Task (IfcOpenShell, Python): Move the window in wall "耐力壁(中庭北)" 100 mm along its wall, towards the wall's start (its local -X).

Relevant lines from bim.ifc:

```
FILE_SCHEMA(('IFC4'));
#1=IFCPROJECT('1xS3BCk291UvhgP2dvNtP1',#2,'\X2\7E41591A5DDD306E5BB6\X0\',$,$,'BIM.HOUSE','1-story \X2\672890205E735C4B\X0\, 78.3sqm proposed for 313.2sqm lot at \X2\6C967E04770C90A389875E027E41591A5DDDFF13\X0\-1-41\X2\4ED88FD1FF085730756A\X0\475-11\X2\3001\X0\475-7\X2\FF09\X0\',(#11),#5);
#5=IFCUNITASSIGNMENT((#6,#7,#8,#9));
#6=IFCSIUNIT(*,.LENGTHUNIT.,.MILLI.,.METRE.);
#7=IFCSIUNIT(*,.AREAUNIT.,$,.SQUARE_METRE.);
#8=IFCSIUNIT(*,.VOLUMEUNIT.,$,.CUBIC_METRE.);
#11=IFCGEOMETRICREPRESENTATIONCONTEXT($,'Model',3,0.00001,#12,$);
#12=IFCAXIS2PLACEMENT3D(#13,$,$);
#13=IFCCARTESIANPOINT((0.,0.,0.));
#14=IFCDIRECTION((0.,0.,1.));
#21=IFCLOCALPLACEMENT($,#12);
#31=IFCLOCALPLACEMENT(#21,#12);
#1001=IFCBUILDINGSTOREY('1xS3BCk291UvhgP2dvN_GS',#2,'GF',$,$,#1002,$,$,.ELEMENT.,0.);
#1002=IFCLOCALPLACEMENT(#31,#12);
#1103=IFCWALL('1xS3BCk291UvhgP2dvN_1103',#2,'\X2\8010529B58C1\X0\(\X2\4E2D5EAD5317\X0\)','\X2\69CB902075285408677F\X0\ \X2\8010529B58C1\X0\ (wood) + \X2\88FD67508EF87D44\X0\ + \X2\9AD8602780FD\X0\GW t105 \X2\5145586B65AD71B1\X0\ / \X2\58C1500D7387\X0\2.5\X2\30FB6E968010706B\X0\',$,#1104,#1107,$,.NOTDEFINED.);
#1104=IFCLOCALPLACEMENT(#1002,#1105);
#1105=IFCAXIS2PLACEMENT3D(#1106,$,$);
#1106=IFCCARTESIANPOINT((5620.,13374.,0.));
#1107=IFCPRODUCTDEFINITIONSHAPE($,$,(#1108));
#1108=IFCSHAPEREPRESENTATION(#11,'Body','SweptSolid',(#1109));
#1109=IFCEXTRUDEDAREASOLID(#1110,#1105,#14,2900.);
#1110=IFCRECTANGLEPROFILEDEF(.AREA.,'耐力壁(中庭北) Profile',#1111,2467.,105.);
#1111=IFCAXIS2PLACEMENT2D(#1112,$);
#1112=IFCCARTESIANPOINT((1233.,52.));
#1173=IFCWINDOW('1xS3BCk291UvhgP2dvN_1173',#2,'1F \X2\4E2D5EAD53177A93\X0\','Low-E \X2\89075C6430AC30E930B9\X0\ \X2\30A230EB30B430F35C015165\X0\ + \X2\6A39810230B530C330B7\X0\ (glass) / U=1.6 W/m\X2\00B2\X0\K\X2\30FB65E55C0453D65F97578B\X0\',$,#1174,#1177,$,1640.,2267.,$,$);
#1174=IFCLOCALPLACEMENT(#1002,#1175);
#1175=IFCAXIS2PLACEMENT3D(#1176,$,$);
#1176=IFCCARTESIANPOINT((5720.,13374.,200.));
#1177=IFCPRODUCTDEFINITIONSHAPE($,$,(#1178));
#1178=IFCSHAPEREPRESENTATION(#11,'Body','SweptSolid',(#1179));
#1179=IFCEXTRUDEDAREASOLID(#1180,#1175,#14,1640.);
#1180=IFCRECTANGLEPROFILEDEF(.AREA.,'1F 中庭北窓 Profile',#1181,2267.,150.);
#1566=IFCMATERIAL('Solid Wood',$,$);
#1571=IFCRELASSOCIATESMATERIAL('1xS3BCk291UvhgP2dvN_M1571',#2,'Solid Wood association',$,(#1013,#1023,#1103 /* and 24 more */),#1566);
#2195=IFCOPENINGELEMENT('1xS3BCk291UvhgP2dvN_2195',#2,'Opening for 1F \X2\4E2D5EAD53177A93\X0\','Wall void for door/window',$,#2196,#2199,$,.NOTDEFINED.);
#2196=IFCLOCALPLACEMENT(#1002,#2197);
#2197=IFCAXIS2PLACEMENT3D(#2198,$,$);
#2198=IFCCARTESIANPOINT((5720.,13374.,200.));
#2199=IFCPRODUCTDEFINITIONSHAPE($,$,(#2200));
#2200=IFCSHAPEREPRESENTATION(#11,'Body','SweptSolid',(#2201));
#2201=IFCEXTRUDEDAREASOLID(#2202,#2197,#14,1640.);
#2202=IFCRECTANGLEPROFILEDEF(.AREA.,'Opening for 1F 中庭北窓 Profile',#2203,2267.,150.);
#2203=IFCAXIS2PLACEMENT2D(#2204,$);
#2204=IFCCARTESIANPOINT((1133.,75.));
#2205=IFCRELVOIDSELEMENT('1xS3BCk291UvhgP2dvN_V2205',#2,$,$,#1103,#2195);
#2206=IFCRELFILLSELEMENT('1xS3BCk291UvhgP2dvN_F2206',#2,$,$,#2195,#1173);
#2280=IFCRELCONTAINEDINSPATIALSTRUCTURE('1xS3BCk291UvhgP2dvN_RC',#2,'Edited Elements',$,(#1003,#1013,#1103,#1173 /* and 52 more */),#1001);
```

```python
import ifcopenshell
import ifcopenshell.api.geometry
import ifcopenshell.util.placement
import ifcopenshell.util.unit

model = ifcopenshell.open("bim.ifc")
unit_scale = ifcopenshell.util.unit.calculate_unit_scale(model)

window = model.by_id(1173)
opening = window.FillsVoids[0].RelatingOpeningElement
wall = opening.VoidsElements[0].RelatingBuildingElement

wall_matrix = ifcopenshell.util.placement.get_local_placement(wall.ObjectPlacement)
shift = wall_matrix[:3, 0] * -0.1 / unit_scale
before = ifcopenshell.util.placement.get_local_placement(window.ObjectPlacement)[:3, 3].copy()

# The window is not placed relative to its opening, so move both.
for product in (opening, window):
    matrix = ifcopenshell.util.placement.get_local_placement(product.ObjectPlacement)
    matrix[:3, 3] += shift
    ifcopenshell.api.geometry.edit_object_placement(model, product=product, matrix=matrix, is_si=False)

after = ifcopenshell.util.placement.get_local_placement(window.ObjectPlacement)[:3, 3]
print("window moved by", (after - before).round(3) + 0.0)

model.write("bim_updated.ifc")
```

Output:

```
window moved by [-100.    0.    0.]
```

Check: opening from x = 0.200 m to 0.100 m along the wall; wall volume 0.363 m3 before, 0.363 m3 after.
